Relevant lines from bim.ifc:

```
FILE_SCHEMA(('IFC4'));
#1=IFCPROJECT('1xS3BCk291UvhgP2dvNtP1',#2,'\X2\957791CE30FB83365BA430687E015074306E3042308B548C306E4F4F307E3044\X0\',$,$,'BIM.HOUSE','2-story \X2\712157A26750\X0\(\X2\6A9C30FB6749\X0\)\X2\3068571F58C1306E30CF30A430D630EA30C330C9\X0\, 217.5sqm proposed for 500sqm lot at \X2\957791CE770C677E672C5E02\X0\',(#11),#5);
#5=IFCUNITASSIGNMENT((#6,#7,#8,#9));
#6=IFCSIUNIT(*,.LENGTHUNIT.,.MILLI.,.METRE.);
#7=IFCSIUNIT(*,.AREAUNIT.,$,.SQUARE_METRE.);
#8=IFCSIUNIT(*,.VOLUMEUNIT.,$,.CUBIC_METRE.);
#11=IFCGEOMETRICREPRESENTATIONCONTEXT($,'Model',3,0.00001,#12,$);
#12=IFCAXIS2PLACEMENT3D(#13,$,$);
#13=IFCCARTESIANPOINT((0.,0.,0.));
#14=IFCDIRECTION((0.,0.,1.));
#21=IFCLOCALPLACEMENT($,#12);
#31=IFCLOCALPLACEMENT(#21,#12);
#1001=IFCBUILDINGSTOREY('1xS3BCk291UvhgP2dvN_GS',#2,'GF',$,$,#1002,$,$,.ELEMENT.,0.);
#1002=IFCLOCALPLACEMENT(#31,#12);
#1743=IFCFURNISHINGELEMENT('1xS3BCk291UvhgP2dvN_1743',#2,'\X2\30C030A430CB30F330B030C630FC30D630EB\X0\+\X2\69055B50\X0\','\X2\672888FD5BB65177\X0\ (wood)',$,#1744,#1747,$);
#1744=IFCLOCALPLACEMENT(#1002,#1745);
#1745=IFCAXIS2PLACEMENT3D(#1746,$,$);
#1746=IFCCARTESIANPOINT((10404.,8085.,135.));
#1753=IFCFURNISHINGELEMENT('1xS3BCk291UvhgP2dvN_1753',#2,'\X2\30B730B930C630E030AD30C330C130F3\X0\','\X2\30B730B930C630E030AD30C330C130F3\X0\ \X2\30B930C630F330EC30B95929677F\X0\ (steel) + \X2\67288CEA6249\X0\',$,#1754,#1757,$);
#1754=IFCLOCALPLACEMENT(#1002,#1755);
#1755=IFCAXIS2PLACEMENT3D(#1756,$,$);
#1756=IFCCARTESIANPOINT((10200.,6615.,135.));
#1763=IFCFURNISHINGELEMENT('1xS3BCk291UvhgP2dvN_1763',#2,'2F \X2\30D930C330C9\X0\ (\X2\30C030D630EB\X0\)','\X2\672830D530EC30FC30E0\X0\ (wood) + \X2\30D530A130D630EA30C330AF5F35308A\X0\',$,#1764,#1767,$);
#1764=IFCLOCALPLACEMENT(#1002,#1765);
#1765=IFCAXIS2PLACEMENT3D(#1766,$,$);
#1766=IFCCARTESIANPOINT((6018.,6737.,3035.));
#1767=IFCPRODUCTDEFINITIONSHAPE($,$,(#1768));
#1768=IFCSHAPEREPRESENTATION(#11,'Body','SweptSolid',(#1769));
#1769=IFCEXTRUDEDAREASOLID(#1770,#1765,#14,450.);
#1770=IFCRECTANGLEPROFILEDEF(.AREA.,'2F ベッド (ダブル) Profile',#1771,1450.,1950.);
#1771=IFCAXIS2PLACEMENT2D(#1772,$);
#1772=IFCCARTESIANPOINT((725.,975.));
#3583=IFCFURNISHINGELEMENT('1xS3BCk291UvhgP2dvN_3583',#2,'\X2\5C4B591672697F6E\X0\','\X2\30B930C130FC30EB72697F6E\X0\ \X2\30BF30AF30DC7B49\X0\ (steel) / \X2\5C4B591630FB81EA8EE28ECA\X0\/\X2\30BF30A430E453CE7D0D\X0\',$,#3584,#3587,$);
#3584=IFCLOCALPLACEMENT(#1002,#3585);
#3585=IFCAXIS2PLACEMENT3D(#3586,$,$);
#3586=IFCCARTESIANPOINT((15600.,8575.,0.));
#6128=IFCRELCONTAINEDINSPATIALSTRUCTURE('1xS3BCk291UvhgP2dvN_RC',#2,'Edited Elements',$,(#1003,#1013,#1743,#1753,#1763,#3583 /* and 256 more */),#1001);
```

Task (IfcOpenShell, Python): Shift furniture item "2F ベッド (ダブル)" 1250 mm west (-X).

```python
import ifcopenshell
import ifcopenshell.api.geometry
import ifcopenshell.util.placement
import ifcopenshell.util.unit

model = ifcopenshell.open("bim.ifc")
unit_scale = ifcopenshell.util.unit.calculate_unit_scale(model)

item = model.by_guid("1xS3BCk291UvhgP2dvN_1763")
matrix = ifcopenshell.util.placement.get_local_placement(item.ObjectPlacement)
matrix[0, 3] -= 1.25 / unit_scale
ifcopenshell.api.geometry.edit_object_placement(model, product=item, matrix=matrix, is_si=False)

print(ifcopenshell.util.placement.get_local_placement(item.ObjectPlacement).round(3) + 0.0)

model.write("bim_v2.ifc")
```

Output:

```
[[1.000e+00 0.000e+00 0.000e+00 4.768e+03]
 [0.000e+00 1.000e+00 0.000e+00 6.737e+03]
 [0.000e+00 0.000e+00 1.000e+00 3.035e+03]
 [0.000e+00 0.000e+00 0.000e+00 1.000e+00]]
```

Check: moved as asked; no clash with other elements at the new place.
